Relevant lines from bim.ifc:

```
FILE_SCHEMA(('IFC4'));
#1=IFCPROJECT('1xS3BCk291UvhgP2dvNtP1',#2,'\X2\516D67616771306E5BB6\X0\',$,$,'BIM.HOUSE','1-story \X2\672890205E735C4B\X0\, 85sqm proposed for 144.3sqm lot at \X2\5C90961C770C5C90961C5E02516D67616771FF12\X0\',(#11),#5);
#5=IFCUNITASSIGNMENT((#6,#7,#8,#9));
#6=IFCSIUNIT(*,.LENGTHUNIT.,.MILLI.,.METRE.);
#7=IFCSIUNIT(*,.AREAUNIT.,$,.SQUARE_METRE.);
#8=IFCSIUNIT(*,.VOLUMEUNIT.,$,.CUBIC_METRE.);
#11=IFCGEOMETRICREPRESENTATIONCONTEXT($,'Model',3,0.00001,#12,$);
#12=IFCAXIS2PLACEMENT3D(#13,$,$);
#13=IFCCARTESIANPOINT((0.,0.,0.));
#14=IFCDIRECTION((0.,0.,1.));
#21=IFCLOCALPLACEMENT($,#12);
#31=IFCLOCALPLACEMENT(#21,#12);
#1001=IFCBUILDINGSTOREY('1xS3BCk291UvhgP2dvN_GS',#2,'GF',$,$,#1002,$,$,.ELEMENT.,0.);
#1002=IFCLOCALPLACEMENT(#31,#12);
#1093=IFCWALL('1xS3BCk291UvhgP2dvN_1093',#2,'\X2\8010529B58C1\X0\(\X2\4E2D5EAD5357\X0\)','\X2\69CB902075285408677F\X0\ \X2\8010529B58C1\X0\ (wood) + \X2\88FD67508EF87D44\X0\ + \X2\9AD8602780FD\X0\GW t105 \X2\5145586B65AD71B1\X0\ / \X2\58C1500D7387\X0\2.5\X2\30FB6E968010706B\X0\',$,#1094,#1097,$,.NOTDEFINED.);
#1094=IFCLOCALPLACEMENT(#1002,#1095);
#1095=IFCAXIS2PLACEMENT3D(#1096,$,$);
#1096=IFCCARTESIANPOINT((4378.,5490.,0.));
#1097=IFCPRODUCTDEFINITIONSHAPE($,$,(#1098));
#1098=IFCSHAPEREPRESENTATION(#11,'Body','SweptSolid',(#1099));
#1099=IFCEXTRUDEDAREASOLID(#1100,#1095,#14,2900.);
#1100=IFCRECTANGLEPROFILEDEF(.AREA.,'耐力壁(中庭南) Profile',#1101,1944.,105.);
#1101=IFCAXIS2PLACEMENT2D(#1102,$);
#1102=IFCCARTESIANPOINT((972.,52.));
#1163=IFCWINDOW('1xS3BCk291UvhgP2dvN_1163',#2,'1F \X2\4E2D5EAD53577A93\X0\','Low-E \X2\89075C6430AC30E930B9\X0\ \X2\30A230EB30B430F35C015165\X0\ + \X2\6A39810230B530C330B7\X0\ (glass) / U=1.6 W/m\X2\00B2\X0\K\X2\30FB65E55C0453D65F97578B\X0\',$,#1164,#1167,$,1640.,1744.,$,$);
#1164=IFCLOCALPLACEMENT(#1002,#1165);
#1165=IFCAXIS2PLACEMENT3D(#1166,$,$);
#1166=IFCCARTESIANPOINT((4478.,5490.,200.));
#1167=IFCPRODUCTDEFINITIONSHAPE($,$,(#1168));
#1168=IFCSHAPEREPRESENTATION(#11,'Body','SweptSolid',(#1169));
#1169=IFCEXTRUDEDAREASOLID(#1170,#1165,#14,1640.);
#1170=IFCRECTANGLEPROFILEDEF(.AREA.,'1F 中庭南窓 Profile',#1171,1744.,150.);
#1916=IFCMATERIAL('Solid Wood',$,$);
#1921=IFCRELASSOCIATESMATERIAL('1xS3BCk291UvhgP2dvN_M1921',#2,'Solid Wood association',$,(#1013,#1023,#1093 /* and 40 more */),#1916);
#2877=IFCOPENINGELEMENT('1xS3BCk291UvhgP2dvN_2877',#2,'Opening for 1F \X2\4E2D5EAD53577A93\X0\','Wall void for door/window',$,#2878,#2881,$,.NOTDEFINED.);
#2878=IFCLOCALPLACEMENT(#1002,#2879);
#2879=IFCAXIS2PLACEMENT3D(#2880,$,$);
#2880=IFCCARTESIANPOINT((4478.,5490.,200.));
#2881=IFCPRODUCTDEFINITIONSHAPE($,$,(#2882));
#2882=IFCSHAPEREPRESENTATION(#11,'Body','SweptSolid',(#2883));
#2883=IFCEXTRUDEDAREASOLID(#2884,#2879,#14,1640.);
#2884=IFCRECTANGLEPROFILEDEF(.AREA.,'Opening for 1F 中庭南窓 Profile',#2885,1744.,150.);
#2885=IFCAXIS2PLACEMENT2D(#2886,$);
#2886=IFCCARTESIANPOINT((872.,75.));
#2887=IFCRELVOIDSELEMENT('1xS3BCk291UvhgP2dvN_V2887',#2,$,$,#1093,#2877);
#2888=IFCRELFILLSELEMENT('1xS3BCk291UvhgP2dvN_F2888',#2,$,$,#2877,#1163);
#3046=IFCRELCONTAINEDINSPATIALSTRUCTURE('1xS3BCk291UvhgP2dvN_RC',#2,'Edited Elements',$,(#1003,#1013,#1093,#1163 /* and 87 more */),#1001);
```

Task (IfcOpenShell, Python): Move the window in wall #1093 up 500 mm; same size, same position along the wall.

```python
import numpy as np
import ifcopenshell
import ifcopenshell.api.geometry
import ifcopenshell.util.placement
import ifcopenshell.util.unit

model = ifcopenshell.open("bim.ifc")
unit_scale = ifcopenshell.util.unit.calculate_unit_scale(model)

window = model.by_id(1163)
opening = window.FillsVoids[0].RelatingOpeningElement
dz = 0.5 / unit_scale

shift = np.array([0.0, 0.0, dz])
# The window is not placed relative to its opening, so move both.
for product in (opening, window):
    matrix = ifcopenshell.util.placement.get_local_placement(product.ObjectPlacement)
    matrix[:3, 3] += shift
    ifcopenshell.api.geometry.edit_object_placement(model, product=product, matrix=matrix, is_si=False)

print(f"moved by {dz * unit_scale:+.3f} m")

model.write("bim_v2.ifc")
```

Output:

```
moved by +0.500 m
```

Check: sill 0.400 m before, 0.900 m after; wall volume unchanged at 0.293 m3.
